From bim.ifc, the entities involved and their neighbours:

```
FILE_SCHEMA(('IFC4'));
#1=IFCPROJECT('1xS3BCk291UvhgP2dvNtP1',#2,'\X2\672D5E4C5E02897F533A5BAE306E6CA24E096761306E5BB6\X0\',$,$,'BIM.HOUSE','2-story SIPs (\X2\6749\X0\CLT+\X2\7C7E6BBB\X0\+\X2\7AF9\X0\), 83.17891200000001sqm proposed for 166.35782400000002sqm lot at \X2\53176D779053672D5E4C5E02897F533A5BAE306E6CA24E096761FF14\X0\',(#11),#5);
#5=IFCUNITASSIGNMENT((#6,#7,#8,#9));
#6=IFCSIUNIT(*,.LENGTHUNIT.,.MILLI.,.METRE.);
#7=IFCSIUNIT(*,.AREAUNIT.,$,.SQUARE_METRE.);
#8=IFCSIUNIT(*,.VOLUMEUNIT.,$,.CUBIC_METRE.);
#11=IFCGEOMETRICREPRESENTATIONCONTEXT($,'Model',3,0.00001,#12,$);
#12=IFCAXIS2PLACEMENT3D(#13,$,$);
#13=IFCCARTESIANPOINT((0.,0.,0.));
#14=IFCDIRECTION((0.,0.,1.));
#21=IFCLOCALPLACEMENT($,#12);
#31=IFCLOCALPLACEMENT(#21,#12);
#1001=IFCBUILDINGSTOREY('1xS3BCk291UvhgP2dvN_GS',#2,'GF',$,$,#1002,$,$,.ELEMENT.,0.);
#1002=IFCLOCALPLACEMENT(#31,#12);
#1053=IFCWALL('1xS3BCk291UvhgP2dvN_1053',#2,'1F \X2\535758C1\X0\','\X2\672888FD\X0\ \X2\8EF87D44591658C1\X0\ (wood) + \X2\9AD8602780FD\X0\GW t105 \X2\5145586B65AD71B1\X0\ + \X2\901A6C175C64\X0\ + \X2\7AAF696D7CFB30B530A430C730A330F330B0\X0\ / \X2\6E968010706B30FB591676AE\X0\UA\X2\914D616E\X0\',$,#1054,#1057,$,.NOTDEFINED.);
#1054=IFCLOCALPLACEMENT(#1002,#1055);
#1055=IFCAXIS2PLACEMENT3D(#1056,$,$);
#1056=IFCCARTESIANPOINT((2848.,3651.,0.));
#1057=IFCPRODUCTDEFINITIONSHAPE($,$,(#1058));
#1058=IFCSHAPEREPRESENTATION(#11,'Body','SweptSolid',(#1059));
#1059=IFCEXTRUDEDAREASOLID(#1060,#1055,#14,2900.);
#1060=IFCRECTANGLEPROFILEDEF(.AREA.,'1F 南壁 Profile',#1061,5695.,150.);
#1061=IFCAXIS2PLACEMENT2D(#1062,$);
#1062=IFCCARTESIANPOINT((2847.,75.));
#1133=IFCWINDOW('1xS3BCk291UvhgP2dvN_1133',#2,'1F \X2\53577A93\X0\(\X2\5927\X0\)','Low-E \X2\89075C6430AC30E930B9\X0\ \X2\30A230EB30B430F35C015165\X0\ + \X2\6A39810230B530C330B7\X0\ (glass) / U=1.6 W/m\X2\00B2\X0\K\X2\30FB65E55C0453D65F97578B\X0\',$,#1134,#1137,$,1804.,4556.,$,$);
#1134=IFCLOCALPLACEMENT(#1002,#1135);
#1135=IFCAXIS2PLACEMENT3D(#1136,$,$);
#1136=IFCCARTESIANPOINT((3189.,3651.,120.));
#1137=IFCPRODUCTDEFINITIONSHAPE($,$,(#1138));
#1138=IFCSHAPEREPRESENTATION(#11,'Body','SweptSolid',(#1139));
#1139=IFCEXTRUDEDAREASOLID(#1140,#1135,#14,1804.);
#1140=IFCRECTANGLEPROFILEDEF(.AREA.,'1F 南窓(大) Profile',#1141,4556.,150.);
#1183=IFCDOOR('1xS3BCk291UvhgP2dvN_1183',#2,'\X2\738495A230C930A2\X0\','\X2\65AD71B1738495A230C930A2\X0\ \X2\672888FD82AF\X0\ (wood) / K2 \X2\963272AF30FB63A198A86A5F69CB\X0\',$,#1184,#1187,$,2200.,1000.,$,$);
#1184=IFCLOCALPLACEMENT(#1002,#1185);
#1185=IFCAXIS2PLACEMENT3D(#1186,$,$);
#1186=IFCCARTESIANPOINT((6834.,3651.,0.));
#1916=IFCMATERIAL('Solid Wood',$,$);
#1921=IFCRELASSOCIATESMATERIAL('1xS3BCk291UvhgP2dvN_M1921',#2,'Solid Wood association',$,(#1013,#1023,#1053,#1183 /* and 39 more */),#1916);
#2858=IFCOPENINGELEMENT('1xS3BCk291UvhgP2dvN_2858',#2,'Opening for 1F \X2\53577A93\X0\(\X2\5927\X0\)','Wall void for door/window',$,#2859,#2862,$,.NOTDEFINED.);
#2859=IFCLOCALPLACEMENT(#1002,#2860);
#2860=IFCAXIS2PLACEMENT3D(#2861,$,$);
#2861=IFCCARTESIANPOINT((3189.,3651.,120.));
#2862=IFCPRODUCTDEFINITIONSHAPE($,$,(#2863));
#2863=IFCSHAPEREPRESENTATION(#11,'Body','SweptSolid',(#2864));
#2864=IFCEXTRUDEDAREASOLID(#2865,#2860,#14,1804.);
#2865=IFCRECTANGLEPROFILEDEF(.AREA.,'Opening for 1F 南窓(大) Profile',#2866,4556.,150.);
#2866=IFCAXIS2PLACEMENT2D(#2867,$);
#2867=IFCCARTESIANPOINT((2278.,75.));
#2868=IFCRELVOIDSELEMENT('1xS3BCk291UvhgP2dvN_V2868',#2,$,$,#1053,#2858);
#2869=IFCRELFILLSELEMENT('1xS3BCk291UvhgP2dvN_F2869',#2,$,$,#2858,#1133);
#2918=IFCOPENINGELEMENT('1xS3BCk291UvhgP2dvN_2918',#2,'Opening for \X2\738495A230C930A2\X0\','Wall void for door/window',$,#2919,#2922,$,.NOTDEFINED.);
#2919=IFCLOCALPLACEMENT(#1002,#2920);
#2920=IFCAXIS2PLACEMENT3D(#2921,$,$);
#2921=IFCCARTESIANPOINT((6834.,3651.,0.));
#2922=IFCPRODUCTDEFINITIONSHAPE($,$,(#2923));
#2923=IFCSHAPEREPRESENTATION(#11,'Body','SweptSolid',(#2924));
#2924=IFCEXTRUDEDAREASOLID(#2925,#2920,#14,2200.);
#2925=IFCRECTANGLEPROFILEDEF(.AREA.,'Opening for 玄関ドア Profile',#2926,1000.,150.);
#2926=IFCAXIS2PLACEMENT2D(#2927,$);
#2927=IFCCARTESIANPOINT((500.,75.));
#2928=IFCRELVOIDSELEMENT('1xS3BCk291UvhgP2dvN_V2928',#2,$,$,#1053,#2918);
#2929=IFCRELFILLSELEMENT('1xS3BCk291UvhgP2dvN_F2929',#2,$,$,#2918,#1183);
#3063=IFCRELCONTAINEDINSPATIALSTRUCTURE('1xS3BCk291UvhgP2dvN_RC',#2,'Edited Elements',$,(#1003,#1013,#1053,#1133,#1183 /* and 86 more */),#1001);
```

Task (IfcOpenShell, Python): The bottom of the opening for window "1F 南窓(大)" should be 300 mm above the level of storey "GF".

```python
import numpy as np
import ifcopenshell
import ifcopenshell.api.geometry
import ifcopenshell.geom
import ifcopenshell.util.element
import ifcopenshell.util.placement
import ifcopenshell.util.shape
import ifcopenshell.util.unit

model = ifcopenshell.open("bim.ifc")
unit_scale = ifcopenshell.util.unit.calculate_unit_scale(model)

window = model.by_id(1133)
opening = window.FillsVoids[0].RelatingOpeningElement
storey = ifcopenshell.util.element.get_container(window, ifc_class="IfcBuildingStorey")
level = ifcopenshell.util.placement.get_local_placement(storey.ObjectPlacement)[2, 3]

# The opening's origin need not be at the sill, so measure its lowest point.
shape = ifcopenshell.geom.create_shape(ifcopenshell.geom.settings(), opening)
bottom = ifcopenshell.util.shape.get_shape_bottom_elevation(shape, shape.geometry) / unit_scale
dz = level + 0.3 / unit_scale - bottom

shift = np.array([0.0, 0.0, dz])
# The window is not placed relative to its opening, so move both.
for product in (opening, window):
    matrix = ifcopenshell.util.placement.get_local_placement(product.ObjectPlacement)
    matrix[:3, 3] += shift
    ifcopenshell.api.geometry.edit_object_placement(model, product=product, matrix=matrix, is_si=False)

print(f"moved by {dz * unit_scale:+.3f} m")

model.write("bim_rev.ifc")
```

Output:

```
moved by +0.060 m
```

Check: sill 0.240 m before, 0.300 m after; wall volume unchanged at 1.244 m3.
